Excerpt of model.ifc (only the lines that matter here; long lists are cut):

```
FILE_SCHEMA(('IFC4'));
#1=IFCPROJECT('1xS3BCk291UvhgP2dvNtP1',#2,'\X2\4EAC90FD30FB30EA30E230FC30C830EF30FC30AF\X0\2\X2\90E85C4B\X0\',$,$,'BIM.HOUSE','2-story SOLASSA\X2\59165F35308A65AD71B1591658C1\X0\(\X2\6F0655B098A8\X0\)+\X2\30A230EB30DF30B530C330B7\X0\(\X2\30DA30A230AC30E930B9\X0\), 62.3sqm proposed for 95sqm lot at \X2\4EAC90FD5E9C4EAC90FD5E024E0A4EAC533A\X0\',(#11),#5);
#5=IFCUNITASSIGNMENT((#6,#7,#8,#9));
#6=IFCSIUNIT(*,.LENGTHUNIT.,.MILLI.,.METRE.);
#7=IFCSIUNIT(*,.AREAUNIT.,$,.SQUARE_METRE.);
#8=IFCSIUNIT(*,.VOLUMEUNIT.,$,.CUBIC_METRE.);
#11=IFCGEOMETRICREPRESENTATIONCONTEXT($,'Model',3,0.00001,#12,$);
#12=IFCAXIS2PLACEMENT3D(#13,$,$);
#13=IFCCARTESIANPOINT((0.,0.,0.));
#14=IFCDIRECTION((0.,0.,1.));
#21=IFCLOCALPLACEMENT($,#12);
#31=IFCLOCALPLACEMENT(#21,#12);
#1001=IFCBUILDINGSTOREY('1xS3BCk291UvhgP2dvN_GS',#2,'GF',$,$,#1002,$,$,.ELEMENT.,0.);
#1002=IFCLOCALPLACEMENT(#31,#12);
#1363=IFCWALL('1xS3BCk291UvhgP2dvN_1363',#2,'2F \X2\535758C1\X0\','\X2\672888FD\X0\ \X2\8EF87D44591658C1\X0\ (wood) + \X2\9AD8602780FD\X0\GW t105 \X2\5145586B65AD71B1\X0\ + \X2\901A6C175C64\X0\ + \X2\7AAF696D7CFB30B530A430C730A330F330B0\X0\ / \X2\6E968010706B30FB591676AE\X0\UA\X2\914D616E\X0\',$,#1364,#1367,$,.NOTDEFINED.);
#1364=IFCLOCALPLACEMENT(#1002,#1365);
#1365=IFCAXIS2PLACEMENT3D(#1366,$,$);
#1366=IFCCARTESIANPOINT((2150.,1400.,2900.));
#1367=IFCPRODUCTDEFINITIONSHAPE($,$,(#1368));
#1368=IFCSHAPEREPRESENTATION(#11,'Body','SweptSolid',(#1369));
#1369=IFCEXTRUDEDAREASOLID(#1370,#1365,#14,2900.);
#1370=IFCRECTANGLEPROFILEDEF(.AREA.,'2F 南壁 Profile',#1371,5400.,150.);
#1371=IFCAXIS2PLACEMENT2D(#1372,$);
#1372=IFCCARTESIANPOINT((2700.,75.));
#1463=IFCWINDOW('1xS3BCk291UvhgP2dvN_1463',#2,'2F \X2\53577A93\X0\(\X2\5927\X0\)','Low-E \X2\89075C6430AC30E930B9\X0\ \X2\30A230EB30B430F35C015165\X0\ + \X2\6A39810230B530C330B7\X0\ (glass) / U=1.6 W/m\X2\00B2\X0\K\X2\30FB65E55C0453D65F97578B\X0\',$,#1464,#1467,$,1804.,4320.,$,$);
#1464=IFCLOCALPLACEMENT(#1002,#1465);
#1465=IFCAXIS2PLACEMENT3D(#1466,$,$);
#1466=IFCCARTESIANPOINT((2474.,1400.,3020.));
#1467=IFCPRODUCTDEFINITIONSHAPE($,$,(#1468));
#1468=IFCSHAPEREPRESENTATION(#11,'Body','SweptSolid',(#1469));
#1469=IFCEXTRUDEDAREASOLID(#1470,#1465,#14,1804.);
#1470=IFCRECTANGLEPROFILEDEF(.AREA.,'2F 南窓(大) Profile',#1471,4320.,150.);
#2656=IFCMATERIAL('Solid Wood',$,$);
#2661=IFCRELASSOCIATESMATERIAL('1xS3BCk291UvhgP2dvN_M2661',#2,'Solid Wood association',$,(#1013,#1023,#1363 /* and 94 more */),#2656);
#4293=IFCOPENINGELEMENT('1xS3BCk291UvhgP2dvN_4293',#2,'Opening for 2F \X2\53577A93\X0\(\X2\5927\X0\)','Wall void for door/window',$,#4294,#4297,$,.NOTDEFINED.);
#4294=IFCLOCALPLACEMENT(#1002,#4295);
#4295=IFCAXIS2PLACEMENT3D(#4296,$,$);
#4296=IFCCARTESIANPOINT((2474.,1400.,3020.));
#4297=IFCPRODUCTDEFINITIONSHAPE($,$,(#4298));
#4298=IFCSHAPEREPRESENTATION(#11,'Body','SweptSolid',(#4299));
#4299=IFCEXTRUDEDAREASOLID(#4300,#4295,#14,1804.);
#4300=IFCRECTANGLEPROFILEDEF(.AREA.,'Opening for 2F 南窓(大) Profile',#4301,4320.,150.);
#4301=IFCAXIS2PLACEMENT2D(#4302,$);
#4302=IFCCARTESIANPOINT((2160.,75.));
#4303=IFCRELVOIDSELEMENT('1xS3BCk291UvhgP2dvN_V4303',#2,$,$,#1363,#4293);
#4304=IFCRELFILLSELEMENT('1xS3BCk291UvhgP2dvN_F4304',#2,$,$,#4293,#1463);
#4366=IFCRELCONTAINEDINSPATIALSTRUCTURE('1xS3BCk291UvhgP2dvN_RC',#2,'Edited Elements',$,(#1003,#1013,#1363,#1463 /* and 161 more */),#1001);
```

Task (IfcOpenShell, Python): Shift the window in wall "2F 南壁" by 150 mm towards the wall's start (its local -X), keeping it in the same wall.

```python
import ifcopenshell
import ifcopenshell.api.geometry
import ifcopenshell.util.placement

model = ifcopenshell.open("model.ifc")

window = model.by_guid("1xS3BCk291UvhgP2dvN_1463")
opening = window.FillsVoids[0].RelatingOpeningElement
wall = opening.VoidsElements[0].RelatingBuildingElement

wall_matrix = ifcopenshell.util.placement.get_local_placement(wall.ObjectPlacement)
shift = wall_matrix[:3, 0] * -150.0
before = ifcopenshell.util.placement.get_local_placement(window.ObjectPlacement)[:3, 3].copy()

# The window is not placed relative to its opening, so move both.
for product in (opening, window):
    matrix = ifcopenshell.util.placement.get_local_placement(product.ObjectPlacement)
    matrix[:3, 3] += shift
    ifcopenshell.api.geometry.edit_object_placement(model, product=product, matrix=matrix, is_si=False)

after = ifcopenshell.util.placement.get_local_placement(window.ObjectPlacement)[:3, 3]
print("window moved by", (after - before).round(3) + 0.0)

model.write("model_v2.ifc")
```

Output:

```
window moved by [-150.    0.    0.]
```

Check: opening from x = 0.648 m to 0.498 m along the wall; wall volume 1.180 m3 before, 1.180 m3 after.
